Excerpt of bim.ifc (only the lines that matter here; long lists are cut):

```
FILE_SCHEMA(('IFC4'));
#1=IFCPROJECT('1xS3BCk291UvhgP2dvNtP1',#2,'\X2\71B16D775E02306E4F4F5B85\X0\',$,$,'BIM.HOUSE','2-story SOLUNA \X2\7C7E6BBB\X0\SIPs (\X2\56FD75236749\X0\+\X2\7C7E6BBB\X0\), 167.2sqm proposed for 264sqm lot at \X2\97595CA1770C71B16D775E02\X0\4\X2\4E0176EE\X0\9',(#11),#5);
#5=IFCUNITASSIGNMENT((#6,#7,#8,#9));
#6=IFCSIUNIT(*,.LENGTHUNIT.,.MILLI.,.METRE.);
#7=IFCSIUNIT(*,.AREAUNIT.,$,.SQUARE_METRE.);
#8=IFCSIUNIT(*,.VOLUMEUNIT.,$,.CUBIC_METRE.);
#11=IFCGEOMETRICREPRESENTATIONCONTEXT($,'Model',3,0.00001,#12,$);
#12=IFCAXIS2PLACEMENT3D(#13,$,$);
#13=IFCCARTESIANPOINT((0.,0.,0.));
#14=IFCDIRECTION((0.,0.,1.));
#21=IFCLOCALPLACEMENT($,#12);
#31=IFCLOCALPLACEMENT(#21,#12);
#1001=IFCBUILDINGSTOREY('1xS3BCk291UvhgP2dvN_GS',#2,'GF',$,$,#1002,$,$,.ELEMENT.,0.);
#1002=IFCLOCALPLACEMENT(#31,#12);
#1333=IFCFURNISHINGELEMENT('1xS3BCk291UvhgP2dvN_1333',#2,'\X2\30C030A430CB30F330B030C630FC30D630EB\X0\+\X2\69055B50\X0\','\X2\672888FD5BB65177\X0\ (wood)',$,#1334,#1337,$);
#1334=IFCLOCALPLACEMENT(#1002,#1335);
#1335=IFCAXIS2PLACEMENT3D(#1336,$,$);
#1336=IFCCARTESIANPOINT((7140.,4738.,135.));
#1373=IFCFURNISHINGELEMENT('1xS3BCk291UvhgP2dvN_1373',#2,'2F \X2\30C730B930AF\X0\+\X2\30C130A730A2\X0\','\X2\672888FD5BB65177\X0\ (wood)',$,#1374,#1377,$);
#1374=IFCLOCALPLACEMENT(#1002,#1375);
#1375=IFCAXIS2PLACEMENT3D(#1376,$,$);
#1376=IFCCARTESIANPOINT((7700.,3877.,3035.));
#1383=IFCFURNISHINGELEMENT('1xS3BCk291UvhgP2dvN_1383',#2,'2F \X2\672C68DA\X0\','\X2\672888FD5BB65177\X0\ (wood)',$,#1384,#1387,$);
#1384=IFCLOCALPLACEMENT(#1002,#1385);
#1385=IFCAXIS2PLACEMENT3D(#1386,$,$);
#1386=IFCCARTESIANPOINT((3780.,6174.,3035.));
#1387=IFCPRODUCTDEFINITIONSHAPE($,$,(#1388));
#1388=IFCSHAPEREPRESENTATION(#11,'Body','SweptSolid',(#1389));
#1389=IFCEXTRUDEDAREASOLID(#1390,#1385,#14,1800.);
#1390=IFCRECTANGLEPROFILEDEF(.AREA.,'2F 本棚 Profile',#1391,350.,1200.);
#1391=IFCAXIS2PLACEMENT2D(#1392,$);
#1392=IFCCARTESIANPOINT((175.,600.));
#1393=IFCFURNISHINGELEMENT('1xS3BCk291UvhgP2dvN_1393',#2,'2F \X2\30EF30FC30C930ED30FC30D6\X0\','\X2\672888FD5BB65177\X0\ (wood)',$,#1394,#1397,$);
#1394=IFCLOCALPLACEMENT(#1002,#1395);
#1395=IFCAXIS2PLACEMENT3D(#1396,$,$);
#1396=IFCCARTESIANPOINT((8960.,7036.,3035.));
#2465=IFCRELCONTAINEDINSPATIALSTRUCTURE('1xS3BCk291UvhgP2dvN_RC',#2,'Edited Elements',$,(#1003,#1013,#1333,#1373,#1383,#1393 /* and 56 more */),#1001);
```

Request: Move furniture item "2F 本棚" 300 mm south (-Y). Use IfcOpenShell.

```python
import ifcopenshell
import ifcopenshell.api.geometry
import ifcopenshell.util.placement

model = ifcopenshell.open("bim.ifc")

item = model.by_guid("1xS3BCk291UvhgP2dvN_1383")
matrix = ifcopenshell.util.placement.get_local_placement(item.ObjectPlacement)
matrix[1, 3] -= 300.0
ifcopenshell.api.geometry.edit_object_placement(model, product=item, matrix=matrix, is_si=False)

print(ifcopenshell.util.placement.get_local_placement(item.ObjectPlacement).round(3) + 0.0)

model.write("bim_updated.ifc")
```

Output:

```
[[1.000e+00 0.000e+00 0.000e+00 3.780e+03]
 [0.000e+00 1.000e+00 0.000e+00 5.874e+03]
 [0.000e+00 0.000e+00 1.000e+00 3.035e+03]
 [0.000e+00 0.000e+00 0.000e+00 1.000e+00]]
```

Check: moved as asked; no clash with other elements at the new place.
